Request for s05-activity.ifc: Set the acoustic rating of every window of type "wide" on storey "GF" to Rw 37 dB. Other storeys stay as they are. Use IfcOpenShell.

First a look at what the model holds.

```python
import ifcopenshell
import ifcopenshell.util.element

model = ifcopenshell.open("s05-activity.ifc")
print(model.schema)
storey = next(s for s in model.by_type("IfcBuildingStorey") if s.Name == "GF")
windows = [e for e in ifcopenshell.util.element.get_decomposition(storey) if e.is_a("IfcWindow")]
seen = {}
for e in windows:
    element_type = ifcopenshell.util.element.get_type(e)
    key = (element_type.Name if element_type != e and element_type else None, ifcopenshell.util.element.get_pset(e, "Pset_WindowCommon", "AcousticRating"))
    seen[key] = seen.get(key, 0) + 1
for (name, value), count in sorted(seen.items(), key=str):
    print(count, "x", name, "|", value)
```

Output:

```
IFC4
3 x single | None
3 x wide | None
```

```python
import ifcopenshell
import ifcopenshell.api.pset
import ifcopenshell.util.element

model = ifcopenshell.open("s05-activity.ifc")

storey = next(s for s in model.by_type("IfcBuildingStorey") if s.Name == "GF")
windows = [e for e in ifcopenshell.util.element.get_decomposition(storey) if e.is_a("IfcWindow")]

count = 0
for e in windows:
    element_type = ifcopenshell.util.element.get_type(e)
    if element_type in (None, e) or element_type.Name != "wide":
        continue
    # add_pset returns the element's existing set when there is one.
    pset = ifcopenshell.api.pset.add_pset(model, product=e, name="Pset_WindowCommon")
    ifcopenshell.api.pset.edit_pset(model, pset=pset, properties={"AcousticRating": "Rw 37 dB"})
    count += 1

print(count, "windows updated")

model.write("s05-activity-out.ifc")
```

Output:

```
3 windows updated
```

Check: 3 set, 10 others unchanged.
